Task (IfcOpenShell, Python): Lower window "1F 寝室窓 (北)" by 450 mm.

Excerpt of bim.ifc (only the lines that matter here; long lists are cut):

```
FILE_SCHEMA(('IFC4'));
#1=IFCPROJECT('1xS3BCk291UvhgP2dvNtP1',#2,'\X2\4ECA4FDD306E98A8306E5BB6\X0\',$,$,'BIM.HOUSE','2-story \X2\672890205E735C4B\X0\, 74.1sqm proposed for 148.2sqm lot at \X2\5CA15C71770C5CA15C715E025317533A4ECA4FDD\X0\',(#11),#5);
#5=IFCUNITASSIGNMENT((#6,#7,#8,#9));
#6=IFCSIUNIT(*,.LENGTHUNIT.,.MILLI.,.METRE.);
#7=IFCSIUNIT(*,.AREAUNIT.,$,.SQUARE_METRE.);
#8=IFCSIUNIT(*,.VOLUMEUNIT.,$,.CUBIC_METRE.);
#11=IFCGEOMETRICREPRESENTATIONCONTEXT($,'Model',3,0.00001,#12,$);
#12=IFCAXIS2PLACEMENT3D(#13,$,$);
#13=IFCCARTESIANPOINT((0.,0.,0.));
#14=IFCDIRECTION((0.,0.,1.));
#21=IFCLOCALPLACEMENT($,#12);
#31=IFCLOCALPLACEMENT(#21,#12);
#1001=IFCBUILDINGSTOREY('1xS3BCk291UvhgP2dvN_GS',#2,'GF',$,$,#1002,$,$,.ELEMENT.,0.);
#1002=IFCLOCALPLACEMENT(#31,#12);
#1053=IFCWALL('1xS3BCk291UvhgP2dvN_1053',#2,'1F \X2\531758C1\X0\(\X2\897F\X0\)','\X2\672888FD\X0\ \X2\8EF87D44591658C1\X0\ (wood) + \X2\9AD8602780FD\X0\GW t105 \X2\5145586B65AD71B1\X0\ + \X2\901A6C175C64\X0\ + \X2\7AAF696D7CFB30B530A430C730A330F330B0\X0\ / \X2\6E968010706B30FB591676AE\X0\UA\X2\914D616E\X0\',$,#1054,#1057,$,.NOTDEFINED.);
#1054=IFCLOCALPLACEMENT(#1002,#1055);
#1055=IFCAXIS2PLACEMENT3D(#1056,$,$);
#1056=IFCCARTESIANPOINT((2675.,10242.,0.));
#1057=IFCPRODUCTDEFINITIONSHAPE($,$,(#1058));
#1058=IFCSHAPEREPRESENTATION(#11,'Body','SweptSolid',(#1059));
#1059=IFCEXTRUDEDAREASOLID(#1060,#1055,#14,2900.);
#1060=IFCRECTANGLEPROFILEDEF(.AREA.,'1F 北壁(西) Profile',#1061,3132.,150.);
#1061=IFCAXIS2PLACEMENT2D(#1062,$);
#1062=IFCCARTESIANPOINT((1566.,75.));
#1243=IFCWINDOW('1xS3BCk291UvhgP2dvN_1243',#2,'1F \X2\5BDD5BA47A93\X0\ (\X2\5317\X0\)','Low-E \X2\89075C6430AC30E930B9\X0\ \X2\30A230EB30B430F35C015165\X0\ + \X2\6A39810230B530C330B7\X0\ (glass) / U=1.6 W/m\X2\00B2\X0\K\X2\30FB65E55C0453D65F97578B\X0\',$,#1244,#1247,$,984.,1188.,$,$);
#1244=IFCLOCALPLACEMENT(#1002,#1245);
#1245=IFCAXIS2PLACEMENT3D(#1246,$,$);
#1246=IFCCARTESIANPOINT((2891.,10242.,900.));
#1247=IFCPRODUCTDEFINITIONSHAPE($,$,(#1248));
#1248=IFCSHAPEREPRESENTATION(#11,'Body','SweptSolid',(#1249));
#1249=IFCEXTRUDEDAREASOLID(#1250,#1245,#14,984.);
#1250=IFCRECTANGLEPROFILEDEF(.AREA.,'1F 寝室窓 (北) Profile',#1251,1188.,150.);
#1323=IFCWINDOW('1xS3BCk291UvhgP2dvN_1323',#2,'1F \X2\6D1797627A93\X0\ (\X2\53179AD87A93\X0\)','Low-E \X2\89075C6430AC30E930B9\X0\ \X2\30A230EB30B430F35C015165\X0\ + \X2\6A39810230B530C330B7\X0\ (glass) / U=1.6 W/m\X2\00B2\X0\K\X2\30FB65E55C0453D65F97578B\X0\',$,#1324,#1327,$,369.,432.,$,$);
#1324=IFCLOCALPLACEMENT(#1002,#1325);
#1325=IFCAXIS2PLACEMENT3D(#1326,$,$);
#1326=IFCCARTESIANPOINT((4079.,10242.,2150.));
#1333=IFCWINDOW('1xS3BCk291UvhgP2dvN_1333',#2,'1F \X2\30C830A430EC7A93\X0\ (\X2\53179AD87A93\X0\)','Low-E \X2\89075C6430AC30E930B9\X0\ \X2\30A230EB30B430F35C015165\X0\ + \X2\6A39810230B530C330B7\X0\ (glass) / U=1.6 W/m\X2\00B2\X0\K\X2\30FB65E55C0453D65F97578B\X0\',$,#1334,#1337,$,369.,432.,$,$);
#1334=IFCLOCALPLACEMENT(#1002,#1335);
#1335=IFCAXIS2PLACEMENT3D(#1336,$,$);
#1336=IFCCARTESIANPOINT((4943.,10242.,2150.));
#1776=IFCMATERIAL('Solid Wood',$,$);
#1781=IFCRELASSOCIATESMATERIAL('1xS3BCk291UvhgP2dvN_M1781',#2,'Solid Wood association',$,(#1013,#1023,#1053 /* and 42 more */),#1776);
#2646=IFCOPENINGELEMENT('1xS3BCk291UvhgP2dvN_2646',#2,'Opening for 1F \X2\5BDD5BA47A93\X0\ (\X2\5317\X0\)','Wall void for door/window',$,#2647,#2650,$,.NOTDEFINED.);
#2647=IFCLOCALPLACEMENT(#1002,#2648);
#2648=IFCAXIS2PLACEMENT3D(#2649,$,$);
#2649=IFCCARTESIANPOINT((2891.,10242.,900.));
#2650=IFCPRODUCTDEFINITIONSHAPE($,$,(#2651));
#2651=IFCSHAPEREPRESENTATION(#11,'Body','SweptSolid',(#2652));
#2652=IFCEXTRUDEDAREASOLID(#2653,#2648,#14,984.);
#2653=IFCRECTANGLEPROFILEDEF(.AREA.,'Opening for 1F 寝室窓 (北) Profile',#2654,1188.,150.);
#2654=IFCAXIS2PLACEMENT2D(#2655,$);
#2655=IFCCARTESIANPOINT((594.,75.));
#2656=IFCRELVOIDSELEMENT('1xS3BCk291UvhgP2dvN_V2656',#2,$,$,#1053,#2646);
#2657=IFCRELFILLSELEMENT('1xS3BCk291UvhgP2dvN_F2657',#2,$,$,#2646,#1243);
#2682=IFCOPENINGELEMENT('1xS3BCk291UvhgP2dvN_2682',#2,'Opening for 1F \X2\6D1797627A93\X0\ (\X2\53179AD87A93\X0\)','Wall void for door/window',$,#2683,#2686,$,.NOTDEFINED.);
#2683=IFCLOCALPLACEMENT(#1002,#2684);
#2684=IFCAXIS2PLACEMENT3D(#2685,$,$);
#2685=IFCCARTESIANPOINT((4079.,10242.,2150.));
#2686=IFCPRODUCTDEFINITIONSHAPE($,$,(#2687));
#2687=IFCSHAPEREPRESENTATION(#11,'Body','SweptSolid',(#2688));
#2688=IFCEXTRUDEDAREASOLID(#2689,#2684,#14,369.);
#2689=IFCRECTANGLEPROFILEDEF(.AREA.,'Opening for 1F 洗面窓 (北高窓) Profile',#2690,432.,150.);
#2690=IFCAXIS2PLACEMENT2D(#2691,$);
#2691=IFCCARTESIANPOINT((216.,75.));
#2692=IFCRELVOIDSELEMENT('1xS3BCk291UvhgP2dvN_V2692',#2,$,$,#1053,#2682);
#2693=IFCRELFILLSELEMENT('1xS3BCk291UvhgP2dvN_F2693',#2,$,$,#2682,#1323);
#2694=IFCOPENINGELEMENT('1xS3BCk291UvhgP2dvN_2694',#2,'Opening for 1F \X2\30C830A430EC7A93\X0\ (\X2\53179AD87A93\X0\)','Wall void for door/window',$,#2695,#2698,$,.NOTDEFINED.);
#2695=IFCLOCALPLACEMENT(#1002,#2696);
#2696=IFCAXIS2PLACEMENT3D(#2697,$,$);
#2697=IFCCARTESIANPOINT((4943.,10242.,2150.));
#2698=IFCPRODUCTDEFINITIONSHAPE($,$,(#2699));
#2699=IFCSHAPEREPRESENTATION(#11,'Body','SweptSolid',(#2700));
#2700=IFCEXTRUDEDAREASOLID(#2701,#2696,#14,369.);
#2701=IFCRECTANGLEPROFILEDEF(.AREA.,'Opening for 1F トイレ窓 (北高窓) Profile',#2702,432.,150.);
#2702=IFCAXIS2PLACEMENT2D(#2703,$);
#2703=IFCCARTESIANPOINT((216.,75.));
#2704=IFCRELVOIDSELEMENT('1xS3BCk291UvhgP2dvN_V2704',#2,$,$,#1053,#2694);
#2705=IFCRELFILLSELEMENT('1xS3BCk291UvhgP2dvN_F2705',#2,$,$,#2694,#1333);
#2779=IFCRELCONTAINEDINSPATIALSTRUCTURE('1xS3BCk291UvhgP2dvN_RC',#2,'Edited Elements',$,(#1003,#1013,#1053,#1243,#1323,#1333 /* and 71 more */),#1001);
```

```python
import numpy as np
import ifcopenshell
import ifcopenshell.api.geometry
import ifcopenshell.util.placement
import ifcopenshell.util.unit

model = ifcopenshell.open("bim.ifc")
unit_scale = ifcopenshell.util.unit.calculate_unit_scale(model)

window = model.by_guid("1xS3BCk291UvhgP2dvN_1243")
opening = window.FillsVoids[0].RelatingOpeningElement
dz = -450.0

shift = np.array([0.0, 0.0, dz])
# The window is not placed relative to its opening, so move both.
for product in (opening, window):
    matrix = ifcopenshell.util.placement.get_local_placement(product.ObjectPlacement)
    matrix[:3, 3] += shift
    ifcopenshell.api.geometry.edit_object_placement(model, product=product, matrix=matrix, is_si=False)

print(f"moved by {dz * unit_scale:+.3f} m")

model.write("bim_edited.ifc")
```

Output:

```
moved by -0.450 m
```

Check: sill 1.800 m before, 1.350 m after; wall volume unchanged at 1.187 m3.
